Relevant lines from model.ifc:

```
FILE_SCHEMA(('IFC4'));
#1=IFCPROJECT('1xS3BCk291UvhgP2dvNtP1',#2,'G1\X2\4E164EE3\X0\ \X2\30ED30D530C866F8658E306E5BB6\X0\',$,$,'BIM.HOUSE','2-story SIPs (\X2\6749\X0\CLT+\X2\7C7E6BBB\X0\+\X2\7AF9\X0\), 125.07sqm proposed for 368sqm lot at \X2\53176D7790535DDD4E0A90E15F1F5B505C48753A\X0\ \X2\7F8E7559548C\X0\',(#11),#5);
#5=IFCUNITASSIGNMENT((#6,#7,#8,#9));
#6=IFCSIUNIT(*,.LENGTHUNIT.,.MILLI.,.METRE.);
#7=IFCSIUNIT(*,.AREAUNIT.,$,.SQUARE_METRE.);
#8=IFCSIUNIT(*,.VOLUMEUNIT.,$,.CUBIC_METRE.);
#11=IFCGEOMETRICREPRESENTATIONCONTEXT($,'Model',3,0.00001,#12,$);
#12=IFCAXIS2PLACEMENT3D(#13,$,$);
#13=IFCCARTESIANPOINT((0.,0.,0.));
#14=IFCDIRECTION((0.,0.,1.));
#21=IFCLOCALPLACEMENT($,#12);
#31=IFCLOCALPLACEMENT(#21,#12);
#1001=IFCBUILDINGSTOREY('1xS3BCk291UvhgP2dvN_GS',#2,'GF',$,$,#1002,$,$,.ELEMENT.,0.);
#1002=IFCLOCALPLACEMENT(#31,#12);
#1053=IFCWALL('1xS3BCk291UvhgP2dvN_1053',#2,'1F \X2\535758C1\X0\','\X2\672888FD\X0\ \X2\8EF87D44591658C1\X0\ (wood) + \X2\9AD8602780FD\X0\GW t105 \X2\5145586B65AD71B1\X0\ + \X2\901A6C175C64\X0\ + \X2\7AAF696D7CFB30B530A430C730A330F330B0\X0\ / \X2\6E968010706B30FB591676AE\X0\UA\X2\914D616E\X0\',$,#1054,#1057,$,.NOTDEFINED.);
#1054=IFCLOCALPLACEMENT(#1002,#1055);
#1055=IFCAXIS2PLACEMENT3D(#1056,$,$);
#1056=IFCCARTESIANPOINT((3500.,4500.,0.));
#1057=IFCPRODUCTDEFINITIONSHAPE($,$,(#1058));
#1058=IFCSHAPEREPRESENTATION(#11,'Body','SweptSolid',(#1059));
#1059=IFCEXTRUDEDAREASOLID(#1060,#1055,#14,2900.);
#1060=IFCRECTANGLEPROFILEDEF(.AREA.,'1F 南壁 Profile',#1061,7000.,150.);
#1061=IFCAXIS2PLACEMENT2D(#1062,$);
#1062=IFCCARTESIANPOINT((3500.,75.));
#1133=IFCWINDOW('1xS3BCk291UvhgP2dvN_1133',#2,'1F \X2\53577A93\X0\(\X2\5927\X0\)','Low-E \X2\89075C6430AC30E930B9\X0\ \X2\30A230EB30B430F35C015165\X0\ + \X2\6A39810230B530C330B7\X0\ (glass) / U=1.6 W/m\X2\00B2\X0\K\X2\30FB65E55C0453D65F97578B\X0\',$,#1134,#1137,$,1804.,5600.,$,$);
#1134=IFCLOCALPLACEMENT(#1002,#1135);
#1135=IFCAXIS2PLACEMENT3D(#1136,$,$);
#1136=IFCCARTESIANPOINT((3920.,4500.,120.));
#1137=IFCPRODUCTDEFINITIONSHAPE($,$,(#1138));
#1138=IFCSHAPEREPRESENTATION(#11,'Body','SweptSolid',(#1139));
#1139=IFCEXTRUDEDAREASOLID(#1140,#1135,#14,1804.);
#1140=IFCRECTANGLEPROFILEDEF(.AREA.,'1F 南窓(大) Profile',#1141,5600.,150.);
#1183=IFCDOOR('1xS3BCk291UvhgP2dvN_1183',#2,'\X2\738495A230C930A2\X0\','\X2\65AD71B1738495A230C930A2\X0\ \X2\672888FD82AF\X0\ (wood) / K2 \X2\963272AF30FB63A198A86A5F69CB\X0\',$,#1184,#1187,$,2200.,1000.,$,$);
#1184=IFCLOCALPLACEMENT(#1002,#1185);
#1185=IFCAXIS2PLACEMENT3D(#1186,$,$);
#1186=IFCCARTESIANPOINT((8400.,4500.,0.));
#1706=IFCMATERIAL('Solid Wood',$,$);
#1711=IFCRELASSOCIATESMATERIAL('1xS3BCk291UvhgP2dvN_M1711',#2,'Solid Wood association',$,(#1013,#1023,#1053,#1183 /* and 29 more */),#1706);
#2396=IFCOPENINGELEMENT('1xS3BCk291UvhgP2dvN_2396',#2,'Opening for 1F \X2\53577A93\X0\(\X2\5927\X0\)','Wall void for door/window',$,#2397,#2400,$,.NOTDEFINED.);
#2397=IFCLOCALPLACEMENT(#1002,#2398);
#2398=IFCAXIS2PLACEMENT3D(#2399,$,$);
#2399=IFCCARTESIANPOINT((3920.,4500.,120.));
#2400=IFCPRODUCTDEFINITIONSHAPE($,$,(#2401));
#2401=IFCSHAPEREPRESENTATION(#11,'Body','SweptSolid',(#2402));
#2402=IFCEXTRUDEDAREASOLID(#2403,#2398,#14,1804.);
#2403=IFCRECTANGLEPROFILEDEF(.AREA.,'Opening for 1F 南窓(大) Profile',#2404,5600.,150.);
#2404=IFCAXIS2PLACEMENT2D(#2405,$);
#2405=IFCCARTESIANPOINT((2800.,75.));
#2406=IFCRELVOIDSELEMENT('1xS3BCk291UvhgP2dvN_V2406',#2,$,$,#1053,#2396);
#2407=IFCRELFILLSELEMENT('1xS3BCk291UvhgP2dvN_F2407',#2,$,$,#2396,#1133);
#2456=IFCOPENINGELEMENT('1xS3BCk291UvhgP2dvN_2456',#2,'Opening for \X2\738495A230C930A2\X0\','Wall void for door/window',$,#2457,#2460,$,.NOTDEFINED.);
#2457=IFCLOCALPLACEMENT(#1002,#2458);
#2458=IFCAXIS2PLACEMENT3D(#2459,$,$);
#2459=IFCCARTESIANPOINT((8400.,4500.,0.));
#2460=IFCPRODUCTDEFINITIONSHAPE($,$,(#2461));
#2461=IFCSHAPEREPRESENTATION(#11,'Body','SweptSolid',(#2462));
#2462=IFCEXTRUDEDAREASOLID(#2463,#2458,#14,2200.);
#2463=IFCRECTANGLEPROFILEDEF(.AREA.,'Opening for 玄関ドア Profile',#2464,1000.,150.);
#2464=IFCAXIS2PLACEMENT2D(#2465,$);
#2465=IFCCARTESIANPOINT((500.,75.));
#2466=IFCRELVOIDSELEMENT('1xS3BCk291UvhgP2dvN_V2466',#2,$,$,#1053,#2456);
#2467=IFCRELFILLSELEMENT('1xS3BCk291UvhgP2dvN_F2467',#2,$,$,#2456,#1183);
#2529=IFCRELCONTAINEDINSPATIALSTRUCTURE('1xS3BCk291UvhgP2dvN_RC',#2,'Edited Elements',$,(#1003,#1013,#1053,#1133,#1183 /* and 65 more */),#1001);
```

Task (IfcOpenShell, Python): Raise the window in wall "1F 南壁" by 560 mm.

```python
import numpy as np
import ifcopenshell
import ifcopenshell.api.geometry
import ifcopenshell.util.placement
import ifcopenshell.util.unit

model = ifcopenshell.open("model.ifc")
unit_scale = ifcopenshell.util.unit.calculate_unit_scale(model)

window = model.by_guid("1xS3BCk291UvhgP2dvN_1133")
opening = window.FillsVoids[0].RelatingOpeningElement
dz = 560.0

shift = np.array([0.0, 0.0, dz])
# The window is not placed relative to its opening, so move both.
for product in (opening, window):
    matrix = ifcopenshell.util.placement.get_local_placement(product.ObjectPlacement)
    matrix[:3, 3] += shift
    ifcopenshell.api.geometry.edit_object_placement(model, product=product, matrix=matrix, is_si=False)

print(f"moved by {dz * unit_scale:+.3f} m")

model.write("model_edited.ifc")
```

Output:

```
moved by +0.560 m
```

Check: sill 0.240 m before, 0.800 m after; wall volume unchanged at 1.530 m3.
